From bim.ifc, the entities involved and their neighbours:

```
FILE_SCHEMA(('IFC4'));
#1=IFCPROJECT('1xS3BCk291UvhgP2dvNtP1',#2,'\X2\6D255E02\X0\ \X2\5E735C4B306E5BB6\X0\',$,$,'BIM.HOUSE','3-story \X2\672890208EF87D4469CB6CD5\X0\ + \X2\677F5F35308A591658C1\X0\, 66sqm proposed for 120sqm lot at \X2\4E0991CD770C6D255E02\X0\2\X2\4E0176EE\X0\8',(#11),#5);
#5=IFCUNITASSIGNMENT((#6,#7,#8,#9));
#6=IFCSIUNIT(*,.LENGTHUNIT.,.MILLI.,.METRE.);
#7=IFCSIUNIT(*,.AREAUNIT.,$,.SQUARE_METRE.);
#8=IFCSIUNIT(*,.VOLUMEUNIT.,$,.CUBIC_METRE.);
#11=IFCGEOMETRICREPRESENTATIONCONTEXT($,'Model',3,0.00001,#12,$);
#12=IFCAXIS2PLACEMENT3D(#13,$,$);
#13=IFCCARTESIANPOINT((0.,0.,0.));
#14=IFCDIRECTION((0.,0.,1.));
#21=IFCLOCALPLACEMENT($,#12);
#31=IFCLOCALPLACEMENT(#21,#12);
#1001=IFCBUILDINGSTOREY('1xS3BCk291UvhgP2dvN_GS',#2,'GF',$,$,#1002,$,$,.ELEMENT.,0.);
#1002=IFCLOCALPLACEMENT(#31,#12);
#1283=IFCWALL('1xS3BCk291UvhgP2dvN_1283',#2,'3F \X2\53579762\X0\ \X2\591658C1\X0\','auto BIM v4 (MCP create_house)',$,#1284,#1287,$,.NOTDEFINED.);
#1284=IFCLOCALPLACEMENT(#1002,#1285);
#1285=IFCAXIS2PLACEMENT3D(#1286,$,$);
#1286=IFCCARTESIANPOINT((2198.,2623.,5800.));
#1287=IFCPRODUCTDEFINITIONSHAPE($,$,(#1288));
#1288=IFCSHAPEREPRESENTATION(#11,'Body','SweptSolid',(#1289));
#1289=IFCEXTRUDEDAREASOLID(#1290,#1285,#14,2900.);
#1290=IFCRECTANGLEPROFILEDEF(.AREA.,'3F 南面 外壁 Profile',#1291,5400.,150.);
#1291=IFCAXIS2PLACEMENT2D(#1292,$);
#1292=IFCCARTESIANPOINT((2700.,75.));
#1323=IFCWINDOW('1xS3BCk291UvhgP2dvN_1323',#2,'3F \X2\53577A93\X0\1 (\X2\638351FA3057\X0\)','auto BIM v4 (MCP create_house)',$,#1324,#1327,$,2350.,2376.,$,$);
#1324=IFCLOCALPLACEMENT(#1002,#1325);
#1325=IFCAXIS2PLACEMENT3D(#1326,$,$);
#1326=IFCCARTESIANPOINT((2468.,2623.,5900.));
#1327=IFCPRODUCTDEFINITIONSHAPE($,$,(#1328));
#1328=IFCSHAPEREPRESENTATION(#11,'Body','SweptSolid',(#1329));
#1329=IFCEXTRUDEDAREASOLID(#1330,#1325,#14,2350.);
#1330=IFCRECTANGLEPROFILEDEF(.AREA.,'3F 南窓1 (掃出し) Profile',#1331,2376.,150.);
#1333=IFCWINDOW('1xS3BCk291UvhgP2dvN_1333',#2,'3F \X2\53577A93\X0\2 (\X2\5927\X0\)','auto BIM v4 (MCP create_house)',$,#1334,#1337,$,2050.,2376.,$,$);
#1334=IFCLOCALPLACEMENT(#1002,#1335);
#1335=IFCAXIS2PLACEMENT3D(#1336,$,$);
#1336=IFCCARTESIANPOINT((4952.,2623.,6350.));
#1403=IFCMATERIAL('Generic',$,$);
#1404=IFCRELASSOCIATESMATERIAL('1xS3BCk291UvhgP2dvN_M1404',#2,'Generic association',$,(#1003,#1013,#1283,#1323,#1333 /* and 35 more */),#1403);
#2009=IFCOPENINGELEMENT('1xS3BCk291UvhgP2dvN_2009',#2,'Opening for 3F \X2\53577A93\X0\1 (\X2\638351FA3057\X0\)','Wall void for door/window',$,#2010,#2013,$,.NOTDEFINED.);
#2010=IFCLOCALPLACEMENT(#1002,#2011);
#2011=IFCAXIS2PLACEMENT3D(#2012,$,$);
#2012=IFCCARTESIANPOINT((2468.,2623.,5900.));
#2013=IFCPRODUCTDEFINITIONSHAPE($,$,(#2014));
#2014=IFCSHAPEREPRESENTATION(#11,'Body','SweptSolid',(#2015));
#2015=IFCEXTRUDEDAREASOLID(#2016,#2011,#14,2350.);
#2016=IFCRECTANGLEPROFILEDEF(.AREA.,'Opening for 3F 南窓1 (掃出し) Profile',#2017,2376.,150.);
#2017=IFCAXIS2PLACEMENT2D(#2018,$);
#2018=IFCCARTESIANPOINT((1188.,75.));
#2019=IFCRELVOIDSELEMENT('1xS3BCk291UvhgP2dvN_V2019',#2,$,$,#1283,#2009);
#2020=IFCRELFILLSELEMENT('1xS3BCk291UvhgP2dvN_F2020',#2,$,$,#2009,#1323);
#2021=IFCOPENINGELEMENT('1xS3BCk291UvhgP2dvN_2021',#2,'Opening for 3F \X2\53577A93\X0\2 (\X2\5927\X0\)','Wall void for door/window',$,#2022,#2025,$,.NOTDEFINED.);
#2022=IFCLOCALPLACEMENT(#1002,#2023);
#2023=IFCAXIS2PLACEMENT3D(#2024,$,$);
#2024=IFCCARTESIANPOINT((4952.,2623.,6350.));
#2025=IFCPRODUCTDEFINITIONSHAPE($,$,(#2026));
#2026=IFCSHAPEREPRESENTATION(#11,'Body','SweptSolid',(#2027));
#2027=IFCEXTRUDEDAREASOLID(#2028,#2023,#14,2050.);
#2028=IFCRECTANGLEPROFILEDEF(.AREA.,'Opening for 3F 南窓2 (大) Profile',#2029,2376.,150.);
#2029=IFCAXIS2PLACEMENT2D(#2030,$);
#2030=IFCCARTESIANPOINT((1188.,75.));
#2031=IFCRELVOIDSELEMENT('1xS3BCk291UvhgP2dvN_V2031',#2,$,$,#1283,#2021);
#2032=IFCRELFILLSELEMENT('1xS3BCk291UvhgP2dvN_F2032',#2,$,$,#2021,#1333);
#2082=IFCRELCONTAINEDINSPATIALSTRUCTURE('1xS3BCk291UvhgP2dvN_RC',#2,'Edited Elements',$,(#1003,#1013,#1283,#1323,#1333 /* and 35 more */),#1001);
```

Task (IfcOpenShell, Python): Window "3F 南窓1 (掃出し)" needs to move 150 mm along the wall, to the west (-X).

```python
import ifcopenshell
import ifcopenshell.api.geometry
import ifcopenshell.util.placement

model = ifcopenshell.open("bim.ifc")

window = model.by_guid("1xS3BCk291UvhgP2dvN_1323")
opening = window.FillsVoids[0].RelatingOpeningElement
wall = opening.VoidsElements[0].RelatingBuildingElement

wall_matrix = ifcopenshell.util.placement.get_local_placement(wall.ObjectPlacement)
shift = wall_matrix[:3, 0] * -150.0
before = ifcopenshell.util.placement.get_local_placement(window.ObjectPlacement)[:3, 3].copy()

# The window is not placed relative to its opening, so move both.
for product in (opening, window):
    matrix = ifcopenshell.util.placement.get_local_placement(product.ObjectPlacement)
    matrix[:3, 3] += shift
    ifcopenshell.api.geometry.edit_object_placement(model, product=product, matrix=matrix, is_si=False)

after = ifcopenshell.util.placement.get_local_placement(window.ObjectPlacement)[:3, 3]
print("window moved by", (after - before).round(3) + 0.0)

model.write("bim_rev.ifc")
```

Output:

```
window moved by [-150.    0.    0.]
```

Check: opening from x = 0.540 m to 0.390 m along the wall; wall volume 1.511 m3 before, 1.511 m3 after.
